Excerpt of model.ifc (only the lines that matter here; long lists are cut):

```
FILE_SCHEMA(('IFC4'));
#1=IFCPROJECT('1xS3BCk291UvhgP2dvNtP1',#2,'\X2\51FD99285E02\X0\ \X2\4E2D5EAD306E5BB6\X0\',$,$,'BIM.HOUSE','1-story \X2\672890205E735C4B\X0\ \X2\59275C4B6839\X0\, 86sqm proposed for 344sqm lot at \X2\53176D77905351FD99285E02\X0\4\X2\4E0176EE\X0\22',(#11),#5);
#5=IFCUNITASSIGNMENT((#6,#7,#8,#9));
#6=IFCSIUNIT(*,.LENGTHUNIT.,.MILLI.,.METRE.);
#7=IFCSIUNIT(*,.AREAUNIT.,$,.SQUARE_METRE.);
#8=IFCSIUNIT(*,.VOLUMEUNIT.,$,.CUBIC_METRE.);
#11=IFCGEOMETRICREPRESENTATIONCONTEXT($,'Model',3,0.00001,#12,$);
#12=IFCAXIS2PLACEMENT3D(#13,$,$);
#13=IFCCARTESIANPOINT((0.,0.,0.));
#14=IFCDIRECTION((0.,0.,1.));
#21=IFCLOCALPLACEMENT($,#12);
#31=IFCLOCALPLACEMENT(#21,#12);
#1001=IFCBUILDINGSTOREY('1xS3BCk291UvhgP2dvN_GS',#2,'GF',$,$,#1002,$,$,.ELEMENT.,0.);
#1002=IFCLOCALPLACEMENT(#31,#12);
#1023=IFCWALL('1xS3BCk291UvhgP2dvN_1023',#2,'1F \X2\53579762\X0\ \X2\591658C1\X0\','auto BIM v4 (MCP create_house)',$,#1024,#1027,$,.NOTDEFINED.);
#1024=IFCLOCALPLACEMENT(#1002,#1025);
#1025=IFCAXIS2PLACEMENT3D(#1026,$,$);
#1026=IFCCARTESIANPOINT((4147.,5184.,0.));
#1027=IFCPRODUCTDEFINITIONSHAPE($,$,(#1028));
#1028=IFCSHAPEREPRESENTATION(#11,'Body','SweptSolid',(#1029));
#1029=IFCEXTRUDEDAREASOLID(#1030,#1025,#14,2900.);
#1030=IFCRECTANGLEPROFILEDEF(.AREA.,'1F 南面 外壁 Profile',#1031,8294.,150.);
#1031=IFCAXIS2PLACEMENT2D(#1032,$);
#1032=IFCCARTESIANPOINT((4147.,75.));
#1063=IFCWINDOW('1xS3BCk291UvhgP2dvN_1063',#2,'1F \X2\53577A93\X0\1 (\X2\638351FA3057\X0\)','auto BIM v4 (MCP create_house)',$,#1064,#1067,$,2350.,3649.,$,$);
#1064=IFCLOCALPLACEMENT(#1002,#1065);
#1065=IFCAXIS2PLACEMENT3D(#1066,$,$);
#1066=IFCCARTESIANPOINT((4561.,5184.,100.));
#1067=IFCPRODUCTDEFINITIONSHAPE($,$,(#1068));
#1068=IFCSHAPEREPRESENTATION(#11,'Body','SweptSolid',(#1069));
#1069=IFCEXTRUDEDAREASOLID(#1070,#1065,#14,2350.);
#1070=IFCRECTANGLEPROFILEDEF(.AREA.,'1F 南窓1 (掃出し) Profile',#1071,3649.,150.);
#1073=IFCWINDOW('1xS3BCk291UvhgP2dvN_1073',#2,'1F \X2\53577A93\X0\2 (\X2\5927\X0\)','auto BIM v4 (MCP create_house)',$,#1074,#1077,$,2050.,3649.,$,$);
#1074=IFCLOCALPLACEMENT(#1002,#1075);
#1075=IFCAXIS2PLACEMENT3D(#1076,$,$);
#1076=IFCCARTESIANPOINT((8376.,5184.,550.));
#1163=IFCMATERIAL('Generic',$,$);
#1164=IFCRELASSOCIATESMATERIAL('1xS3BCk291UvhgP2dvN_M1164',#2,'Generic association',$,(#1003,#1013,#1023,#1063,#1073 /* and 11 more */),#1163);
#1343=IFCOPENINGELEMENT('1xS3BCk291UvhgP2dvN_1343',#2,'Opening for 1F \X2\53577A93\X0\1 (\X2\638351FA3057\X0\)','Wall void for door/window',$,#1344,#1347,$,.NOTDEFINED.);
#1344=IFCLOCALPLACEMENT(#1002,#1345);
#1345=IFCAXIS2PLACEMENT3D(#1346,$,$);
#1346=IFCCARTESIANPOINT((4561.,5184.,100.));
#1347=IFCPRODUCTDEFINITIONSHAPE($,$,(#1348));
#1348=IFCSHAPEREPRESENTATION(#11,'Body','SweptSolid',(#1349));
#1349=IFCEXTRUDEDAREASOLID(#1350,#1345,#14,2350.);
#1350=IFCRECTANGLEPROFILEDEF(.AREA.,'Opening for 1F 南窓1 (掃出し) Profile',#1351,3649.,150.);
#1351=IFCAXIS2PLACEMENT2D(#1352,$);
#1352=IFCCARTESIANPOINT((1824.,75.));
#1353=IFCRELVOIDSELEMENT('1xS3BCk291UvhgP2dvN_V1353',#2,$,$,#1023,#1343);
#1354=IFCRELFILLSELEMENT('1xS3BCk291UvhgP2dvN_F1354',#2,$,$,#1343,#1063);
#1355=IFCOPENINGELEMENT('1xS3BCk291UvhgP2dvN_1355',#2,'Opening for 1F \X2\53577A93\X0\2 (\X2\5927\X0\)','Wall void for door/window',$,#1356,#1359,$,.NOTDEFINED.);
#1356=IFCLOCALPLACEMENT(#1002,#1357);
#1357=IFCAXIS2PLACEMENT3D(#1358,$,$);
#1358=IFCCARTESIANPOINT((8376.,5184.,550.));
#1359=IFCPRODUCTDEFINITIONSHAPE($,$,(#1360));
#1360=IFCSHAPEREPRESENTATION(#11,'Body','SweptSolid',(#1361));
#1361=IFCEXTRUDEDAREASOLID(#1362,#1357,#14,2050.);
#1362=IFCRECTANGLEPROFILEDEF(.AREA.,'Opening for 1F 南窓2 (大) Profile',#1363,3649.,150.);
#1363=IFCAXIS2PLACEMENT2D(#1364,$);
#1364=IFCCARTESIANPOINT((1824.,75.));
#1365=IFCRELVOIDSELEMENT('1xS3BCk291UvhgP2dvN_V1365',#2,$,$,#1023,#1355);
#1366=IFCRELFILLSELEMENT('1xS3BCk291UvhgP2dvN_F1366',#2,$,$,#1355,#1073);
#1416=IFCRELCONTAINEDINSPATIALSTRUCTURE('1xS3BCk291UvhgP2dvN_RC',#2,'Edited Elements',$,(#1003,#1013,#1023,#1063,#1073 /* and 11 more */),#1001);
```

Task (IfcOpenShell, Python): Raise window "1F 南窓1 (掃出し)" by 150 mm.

```python
import numpy as np
import ifcopenshell
import ifcopenshell.api.geometry
import ifcopenshell.util.placement
import ifcopenshell.util.unit

model = ifcopenshell.open("model.ifc")
unit_scale = ifcopenshell.util.unit.calculate_unit_scale(model)

window = model.by_id(1063)
opening = window.FillsVoids[0].RelatingOpeningElement
dz = 0.15 / unit_scale

shift = np.array([0.0, 0.0, dz])
# The window is not placed relative to its opening, so move both.
for product in (opening, window):
    matrix = ifcopenshell.util.placement.get_local_placement(product.ObjectPlacement)
    matrix[:3, 3] += shift
    ifcopenshell.api.geometry.edit_object_placement(model, product=product, matrix=matrix, is_si=False)

print(f"moved by {dz * unit_scale:+.3f} m")

model.write("model_rev.ifc")
```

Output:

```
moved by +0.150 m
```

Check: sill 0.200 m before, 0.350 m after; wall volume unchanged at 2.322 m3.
